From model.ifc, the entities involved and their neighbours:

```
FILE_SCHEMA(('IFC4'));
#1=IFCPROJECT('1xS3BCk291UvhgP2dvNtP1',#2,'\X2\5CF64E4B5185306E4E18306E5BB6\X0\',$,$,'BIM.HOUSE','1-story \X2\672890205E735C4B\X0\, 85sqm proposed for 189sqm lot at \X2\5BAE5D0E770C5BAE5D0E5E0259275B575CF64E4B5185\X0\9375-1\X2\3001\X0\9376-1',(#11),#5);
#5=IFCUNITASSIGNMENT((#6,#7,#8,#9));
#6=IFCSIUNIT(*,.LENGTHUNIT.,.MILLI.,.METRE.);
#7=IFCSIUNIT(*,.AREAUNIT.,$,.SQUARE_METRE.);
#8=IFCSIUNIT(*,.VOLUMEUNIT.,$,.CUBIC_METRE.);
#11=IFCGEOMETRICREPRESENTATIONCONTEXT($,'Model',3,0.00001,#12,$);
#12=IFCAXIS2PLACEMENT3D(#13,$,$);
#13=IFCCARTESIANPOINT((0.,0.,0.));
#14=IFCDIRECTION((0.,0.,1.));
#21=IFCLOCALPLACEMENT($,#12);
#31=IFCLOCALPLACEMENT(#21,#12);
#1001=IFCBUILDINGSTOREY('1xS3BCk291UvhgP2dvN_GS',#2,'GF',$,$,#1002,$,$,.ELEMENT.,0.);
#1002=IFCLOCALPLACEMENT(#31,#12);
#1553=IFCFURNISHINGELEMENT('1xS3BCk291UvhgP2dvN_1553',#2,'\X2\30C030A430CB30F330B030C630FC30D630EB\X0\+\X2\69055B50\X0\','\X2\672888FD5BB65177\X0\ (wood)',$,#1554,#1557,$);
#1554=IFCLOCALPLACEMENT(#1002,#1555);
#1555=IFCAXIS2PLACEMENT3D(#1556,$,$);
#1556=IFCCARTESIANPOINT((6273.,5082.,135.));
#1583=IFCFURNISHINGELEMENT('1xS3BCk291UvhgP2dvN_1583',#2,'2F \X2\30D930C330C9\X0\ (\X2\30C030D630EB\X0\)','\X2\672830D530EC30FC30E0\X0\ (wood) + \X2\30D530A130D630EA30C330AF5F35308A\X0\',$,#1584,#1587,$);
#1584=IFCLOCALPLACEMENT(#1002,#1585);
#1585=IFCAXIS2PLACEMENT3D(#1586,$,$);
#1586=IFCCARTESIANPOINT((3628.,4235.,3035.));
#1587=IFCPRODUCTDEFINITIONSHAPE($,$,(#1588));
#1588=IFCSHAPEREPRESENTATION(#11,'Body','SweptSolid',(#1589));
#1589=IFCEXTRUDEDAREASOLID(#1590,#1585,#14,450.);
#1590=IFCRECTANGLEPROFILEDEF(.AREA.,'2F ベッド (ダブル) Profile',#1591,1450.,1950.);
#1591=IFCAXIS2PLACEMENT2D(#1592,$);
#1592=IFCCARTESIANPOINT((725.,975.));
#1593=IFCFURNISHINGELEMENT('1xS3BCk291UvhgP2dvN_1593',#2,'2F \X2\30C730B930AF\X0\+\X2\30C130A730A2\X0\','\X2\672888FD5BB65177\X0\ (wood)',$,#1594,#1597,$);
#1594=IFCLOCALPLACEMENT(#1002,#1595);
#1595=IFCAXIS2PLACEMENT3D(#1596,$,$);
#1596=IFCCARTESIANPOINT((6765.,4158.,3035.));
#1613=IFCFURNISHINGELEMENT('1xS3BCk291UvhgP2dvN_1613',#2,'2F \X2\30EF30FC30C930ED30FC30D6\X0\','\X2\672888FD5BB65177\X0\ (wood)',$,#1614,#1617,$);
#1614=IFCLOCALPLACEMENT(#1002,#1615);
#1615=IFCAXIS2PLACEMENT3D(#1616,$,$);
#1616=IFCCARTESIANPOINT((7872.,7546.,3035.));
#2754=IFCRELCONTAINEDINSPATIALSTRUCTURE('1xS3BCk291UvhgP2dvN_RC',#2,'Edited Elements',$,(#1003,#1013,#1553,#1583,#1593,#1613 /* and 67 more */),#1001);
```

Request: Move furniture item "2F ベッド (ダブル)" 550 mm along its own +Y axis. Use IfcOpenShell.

```python
import ifcopenshell
import ifcopenshell.api.geometry
import ifcopenshell.util.placement
import ifcopenshell.util.unit

model = ifcopenshell.open("model.ifc")
unit_scale = ifcopenshell.util.unit.calculate_unit_scale(model)

item = model.by_id(1583)
matrix = ifcopenshell.util.placement.get_local_placement(item.ObjectPlacement)
matrix[:3, 3] += matrix[:3, 1] * 0.55 / unit_scale
ifcopenshell.api.geometry.edit_object_placement(model, product=item, matrix=matrix, is_si=False)

print(ifcopenshell.util.placement.get_local_placement(item.ObjectPlacement).round(3) + 0.0)

model.write("model-out.ifc")
```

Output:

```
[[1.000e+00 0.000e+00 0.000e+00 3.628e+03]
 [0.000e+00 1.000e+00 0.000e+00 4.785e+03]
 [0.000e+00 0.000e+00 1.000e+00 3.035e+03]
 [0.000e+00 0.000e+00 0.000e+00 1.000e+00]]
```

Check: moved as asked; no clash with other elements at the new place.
